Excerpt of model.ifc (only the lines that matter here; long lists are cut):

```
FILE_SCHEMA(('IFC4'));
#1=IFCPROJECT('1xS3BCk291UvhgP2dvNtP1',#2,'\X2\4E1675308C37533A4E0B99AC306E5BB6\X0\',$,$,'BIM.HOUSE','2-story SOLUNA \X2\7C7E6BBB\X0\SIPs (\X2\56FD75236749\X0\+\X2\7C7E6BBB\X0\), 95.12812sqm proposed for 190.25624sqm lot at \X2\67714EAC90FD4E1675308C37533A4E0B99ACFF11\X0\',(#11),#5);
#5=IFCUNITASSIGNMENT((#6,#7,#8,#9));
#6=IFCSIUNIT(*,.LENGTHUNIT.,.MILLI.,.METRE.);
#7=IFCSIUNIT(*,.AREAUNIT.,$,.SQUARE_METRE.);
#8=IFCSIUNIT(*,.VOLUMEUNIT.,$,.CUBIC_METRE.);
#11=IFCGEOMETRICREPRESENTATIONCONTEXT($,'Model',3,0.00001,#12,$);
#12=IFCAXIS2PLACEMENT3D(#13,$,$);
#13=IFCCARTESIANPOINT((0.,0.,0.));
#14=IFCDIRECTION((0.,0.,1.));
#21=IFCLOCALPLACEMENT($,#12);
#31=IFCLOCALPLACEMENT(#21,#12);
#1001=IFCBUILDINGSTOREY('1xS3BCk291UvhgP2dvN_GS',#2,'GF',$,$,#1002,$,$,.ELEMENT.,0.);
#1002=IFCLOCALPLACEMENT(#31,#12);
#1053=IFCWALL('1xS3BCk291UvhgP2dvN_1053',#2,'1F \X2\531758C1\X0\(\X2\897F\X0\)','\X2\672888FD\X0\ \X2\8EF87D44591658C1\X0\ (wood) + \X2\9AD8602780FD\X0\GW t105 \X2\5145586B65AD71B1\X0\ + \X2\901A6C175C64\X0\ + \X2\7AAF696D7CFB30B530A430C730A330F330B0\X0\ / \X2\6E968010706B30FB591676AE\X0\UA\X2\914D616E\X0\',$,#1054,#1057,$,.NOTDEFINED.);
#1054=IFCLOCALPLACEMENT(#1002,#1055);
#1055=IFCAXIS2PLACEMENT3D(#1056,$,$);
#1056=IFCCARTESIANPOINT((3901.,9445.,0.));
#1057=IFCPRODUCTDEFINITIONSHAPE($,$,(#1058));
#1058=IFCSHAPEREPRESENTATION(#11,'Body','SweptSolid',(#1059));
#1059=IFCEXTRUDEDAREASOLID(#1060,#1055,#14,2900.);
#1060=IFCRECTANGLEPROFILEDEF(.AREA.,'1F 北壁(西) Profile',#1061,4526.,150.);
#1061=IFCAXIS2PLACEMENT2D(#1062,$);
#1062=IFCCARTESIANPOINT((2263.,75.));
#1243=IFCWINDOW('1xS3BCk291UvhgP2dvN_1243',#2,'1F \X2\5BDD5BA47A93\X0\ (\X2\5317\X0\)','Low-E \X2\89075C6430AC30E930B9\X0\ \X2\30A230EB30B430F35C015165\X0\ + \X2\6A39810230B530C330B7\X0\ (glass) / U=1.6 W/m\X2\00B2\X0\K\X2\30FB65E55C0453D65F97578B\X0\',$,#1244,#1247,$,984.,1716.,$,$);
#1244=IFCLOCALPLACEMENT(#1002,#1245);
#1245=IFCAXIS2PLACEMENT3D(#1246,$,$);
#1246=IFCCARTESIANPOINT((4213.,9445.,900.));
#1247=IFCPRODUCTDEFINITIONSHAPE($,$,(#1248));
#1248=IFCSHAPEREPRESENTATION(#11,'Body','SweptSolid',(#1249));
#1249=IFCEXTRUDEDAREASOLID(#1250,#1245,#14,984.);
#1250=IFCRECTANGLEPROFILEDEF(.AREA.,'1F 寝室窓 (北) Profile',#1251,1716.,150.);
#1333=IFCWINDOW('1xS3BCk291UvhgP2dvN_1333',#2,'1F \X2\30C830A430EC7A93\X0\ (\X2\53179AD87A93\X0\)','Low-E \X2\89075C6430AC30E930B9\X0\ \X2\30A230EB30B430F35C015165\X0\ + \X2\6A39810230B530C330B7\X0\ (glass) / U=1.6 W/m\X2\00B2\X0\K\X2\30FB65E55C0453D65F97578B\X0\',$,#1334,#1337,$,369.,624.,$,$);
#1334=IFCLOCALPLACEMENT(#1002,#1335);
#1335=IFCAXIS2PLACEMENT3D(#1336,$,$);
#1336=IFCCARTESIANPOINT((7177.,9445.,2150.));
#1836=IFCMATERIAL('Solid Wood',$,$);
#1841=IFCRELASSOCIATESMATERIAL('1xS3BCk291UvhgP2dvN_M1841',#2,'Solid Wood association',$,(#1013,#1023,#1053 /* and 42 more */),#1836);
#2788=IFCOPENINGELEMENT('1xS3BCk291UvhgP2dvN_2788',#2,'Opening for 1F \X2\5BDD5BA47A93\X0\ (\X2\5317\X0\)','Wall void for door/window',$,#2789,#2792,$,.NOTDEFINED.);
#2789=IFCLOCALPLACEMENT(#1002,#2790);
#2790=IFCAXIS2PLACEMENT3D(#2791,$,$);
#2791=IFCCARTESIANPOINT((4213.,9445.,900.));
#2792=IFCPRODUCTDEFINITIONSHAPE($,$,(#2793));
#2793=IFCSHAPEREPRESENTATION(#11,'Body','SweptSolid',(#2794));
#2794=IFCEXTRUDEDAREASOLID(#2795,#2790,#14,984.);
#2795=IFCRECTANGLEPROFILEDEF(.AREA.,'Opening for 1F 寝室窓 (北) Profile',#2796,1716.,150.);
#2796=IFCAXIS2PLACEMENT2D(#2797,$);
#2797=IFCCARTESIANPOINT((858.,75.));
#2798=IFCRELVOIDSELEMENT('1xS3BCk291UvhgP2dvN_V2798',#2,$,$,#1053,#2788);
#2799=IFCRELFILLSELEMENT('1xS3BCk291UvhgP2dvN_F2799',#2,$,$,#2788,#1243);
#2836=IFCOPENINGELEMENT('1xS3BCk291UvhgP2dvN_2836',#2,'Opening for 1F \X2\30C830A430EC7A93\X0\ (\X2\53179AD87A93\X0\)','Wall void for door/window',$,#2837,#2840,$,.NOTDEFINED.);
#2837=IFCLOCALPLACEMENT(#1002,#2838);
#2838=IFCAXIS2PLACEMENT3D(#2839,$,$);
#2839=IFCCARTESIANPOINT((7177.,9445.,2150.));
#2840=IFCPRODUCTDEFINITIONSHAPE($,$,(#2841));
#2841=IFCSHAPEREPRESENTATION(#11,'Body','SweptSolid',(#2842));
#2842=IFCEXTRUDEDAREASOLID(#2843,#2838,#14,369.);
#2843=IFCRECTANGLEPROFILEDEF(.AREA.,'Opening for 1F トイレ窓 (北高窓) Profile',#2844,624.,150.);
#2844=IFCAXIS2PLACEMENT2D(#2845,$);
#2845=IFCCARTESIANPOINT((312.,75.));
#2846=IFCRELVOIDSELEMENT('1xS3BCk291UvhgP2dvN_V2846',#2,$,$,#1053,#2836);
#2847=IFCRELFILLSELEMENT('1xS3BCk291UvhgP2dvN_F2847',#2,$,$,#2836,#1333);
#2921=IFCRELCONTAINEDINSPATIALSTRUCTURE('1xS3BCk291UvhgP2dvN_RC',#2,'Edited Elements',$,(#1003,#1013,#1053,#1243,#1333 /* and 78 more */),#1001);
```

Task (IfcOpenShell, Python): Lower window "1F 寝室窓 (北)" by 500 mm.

```python
import numpy as np
import ifcopenshell
import ifcopenshell.api.geometry
import ifcopenshell.util.placement
import ifcopenshell.util.unit

model = ifcopenshell.open("model.ifc")
unit_scale = ifcopenshell.util.unit.calculate_unit_scale(model)

window = model.by_guid("1xS3BCk291UvhgP2dvN_1243")
opening = window.FillsVoids[0].RelatingOpeningElement
dz = -0.5 / unit_scale

shift = np.array([0.0, 0.0, dz])
# The window is not placed relative to its opening, so move both.
for product in (opening, window):
    matrix = ifcopenshell.util.placement.get_local_placement(product.ObjectPlacement)
    matrix[:3, 3] += shift
    ifcopenshell.api.geometry.edit_object_placement(model, product=product, matrix=matrix, is_si=False)

print(f"moved by {dz * unit_scale:+.3f} m")

model.write("model_v2.ifc")
```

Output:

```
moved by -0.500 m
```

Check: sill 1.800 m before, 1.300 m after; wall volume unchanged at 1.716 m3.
